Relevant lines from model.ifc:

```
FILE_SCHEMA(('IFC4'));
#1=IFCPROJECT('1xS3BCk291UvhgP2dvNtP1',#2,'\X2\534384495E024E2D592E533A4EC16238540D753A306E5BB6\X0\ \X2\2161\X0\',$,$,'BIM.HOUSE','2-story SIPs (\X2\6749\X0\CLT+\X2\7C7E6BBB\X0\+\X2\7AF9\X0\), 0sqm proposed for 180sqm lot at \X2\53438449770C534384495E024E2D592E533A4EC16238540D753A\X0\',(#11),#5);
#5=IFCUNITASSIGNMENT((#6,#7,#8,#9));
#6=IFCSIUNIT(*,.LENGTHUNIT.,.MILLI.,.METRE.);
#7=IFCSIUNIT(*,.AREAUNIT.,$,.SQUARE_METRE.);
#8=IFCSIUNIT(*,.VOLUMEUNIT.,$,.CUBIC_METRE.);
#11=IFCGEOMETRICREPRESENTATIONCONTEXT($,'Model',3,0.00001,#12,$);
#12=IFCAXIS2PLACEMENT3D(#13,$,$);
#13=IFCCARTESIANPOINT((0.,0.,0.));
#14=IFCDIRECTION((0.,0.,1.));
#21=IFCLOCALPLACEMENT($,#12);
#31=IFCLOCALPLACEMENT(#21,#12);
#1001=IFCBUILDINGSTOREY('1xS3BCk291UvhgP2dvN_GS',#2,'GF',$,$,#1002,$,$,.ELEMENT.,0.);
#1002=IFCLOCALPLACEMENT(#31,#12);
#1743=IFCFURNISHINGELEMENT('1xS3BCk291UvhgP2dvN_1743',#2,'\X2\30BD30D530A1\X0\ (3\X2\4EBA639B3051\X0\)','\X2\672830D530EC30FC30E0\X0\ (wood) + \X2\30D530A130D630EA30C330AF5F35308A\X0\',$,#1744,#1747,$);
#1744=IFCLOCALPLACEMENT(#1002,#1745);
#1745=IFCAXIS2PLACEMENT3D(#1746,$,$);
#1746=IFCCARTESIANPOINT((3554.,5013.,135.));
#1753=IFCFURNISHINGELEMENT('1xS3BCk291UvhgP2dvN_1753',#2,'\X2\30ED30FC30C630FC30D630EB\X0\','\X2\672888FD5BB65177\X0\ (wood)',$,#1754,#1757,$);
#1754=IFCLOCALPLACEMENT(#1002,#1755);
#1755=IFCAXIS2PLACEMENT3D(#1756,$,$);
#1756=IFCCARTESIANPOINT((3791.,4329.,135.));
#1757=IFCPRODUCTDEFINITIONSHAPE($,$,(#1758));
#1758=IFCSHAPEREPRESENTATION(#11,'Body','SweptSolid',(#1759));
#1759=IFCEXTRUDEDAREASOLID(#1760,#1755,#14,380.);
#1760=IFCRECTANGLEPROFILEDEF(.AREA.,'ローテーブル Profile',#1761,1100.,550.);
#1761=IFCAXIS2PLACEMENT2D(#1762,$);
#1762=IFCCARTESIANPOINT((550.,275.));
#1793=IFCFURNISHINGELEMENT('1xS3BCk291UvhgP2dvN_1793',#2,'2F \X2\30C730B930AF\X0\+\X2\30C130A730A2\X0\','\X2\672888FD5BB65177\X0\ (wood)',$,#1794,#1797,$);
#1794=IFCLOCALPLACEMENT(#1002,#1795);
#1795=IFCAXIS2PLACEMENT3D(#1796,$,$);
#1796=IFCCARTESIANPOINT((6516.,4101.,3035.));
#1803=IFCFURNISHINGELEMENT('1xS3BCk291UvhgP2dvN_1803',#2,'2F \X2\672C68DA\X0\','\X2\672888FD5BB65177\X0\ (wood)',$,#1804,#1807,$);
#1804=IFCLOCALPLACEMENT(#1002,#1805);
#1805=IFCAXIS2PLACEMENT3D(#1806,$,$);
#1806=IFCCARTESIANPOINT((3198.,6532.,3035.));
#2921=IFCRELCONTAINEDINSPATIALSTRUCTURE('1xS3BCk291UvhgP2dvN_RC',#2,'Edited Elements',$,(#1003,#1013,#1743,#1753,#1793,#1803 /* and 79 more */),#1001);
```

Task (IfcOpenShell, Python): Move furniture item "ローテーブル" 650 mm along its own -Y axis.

```python
import ifcopenshell
import ifcopenshell.api.geometry
import ifcopenshell.util.placement
import ifcopenshell.util.unit

model = ifcopenshell.open("model.ifc")
unit_scale = ifcopenshell.util.unit.calculate_unit_scale(model)

item = model.by_guid("1xS3BCk291UvhgP2dvN_1753")
matrix = ifcopenshell.util.placement.get_local_placement(item.ObjectPlacement)
matrix[:3, 3] -= matrix[:3, 1] * 0.65 / unit_scale
ifcopenshell.api.geometry.edit_object_placement(model, product=item, matrix=matrix, is_si=False)

print(ifcopenshell.util.placement.get_local_placement(item.ObjectPlacement).round(3) + 0.0)

model.write("model_rev.ifc")
```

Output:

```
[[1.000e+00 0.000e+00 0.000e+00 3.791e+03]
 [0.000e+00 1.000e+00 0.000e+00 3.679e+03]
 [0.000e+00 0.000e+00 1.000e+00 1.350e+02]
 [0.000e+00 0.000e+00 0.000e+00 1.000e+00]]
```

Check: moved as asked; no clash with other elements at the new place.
